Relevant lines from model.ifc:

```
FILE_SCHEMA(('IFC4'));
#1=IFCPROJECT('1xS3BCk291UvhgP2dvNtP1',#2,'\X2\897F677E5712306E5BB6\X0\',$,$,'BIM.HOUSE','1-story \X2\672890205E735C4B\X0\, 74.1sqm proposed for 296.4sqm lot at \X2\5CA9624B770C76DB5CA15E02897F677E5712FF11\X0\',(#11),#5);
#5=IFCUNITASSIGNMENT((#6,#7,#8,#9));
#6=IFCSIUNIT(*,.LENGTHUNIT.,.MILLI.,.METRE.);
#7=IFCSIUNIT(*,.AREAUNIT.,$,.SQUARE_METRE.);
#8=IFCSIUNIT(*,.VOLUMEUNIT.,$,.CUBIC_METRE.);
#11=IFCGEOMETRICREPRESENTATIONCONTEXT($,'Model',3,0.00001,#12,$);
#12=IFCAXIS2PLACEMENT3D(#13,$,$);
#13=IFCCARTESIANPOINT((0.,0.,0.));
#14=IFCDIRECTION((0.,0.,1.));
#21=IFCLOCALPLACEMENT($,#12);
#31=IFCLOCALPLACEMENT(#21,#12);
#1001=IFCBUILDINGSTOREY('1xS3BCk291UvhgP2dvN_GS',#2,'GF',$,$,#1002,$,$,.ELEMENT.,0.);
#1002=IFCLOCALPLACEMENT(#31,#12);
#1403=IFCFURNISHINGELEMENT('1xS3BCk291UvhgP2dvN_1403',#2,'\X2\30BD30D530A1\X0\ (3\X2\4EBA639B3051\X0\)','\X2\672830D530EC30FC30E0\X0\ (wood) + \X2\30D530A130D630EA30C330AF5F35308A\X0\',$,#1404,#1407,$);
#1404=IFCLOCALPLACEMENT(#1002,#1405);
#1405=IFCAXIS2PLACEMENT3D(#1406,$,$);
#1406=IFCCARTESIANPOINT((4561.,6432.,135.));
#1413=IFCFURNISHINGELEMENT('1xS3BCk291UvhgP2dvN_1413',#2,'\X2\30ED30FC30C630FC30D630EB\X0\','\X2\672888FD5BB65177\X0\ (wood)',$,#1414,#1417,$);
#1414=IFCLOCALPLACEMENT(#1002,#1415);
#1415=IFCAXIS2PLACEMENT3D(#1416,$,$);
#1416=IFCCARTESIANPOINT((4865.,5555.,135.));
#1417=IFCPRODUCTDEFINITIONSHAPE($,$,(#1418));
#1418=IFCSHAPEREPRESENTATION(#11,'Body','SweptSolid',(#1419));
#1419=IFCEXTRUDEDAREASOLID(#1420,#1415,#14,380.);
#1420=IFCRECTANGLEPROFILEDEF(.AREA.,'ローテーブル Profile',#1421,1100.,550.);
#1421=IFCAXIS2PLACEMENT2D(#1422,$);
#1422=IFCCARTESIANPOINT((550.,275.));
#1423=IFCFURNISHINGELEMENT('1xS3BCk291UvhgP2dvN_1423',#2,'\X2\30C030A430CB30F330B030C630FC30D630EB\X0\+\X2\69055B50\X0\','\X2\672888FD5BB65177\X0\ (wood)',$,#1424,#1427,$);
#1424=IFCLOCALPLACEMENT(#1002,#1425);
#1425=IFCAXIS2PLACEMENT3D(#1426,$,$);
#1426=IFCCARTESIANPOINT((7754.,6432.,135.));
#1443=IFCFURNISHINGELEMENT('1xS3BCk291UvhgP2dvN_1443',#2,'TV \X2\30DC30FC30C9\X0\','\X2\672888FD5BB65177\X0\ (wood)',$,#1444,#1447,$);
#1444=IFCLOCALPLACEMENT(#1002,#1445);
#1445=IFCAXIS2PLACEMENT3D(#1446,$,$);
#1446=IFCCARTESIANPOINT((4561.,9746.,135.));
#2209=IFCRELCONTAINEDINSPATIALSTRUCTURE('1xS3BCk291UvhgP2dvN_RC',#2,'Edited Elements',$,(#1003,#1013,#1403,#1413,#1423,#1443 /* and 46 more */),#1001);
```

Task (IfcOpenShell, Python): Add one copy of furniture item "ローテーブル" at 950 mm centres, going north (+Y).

```python
import numpy as np
import ifcopenshell
import ifcopenshell.api.geometry
import ifcopenshell.api.root
import ifcopenshell.util.element
import ifcopenshell.util.placement
import ifcopenshell.util.unit

model = ifcopenshell.open("model.ifc")
unit_scale = ifcopenshell.util.unit.calculate_unit_scale(model)


def reuse_history(source, copy):
    """copy_class also copies each property set's owner history, people and application; keep the originals."""
    for rel in copy.IsDefinedBy:
        if rel.is_a("IfcRelDefinesByProperties") and (history := rel.RelatingPropertyDefinition.OwnerHistory):
            rel.RelatingPropertyDefinition.OwnerHistory = source.OwnerHistory
            ifcopenshell.util.element.remove_deep2(model, history)


source = model.by_guid("1xS3BCk291UvhgP2dvN_1413")
base = ifcopenshell.util.placement.get_local_placement(source.ObjectPlacement)
step = np.array([0.0, 1.0, 0.0]) * 0.95 / unit_scale

for i in range(1, 2):
    copy = ifcopenshell.api.root.copy_class(model, product=source)
    copy.Representation = ifcopenshell.util.element.copy_deep(
        model, source.Representation, exclude=["IfcGeometricRepresentationContext", "IfcRepresentationMap"]
    )
    reuse_history(source, copy)
    matrix = base.copy()
    matrix[:3, 3] += i * step
    print("added at", matrix[:3, 3].round(3) + 0.0)
    ifcopenshell.api.geometry.edit_object_placement(model, product=copy, matrix=matrix, is_si=False)

model.write("model-out.ifc")
```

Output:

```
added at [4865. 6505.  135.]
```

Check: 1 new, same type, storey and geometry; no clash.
